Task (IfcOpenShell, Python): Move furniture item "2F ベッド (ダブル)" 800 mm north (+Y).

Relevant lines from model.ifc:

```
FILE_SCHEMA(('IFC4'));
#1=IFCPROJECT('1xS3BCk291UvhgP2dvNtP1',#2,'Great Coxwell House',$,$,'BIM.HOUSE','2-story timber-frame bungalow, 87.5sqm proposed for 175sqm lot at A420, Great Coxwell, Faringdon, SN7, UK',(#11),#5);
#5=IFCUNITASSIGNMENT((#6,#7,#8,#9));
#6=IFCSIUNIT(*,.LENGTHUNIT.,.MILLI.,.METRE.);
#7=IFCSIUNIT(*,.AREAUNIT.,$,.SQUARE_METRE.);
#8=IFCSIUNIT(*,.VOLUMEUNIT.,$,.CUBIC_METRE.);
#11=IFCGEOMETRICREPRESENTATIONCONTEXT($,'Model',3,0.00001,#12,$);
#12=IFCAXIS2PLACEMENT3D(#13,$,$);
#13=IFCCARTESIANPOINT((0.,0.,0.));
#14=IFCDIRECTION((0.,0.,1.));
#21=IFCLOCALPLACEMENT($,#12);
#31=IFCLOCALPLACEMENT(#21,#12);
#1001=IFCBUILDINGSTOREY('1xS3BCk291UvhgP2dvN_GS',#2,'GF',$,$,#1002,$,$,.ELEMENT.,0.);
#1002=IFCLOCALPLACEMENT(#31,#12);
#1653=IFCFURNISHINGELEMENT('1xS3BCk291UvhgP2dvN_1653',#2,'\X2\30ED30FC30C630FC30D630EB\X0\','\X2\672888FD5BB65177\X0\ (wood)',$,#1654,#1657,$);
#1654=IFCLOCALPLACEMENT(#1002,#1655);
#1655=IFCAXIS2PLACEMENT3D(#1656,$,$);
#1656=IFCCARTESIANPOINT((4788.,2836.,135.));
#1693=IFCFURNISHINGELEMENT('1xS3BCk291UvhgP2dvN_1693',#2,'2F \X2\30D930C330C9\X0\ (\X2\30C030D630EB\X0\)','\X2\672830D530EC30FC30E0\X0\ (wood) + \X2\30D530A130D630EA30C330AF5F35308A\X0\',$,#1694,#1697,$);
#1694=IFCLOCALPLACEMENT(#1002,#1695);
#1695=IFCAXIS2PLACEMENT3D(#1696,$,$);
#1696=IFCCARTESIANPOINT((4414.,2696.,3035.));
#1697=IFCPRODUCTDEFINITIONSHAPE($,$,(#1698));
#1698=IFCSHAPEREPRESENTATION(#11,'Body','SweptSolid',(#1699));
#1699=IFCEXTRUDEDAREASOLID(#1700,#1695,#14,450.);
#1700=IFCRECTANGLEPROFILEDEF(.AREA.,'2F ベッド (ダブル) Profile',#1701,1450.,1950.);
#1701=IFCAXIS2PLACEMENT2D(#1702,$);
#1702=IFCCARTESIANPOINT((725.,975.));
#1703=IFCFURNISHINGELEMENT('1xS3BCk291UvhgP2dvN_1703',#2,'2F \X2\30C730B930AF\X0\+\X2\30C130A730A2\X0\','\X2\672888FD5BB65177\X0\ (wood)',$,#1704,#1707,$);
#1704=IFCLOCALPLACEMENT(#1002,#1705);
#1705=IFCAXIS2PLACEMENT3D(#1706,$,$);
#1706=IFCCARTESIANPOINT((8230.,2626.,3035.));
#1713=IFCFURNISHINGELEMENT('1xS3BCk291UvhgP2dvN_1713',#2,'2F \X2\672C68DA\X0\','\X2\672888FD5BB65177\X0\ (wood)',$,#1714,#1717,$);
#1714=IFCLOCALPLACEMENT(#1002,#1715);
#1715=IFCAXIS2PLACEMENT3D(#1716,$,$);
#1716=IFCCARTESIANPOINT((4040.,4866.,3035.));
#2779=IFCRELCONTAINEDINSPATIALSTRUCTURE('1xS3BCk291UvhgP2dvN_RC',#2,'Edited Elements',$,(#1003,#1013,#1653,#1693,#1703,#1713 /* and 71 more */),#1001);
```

```python
import ifcopenshell
import ifcopenshell.api.geometry
import ifcopenshell.util.placement

model = ifcopenshell.open("model.ifc")

item = model.by_guid("1xS3BCk291UvhgP2dvN_1693")
matrix = ifcopenshell.util.placement.get_local_placement(item.ObjectPlacement)
matrix[1, 3] += 800.0
ifcopenshell.api.geometry.edit_object_placement(model, product=item, matrix=matrix, is_si=False)

print(ifcopenshell.util.placement.get_local_placement(item.ObjectPlacement).round(3) + 0.0)

model.write("model_v2.ifc")
```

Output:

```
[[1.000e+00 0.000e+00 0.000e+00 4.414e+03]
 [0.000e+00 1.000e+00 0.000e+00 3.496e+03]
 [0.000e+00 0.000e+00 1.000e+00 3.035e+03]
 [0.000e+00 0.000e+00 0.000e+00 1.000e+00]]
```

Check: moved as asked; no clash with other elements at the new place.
